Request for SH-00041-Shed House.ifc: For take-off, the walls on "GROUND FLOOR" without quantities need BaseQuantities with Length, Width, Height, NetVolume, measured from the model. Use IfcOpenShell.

First a look at what the model holds.

```python
import ifcopenshell
import ifcopenshell.util.element
import ifcopenshell.util.unit

model = ifcopenshell.open("SH-00041-Shed House.ifc")
print(model.schema)
for unit_type in ("LENGTHUNIT", "AREAUNIT", "VOLUMEUNIT"):
    print(unit_type, ifcopenshell.util.unit.calculate_unit_scale(model, unit_type))
storey = next(s for s in model.by_type("IfcBuildingStorey") if s.Name == "GROUND FLOOR")
walls = [e for e in ifcopenshell.util.element.get_decomposition(storey) if e.is_a("IfcWall")]
for e in sorted(walls, key=lambda e: e.id()):
    print(e.id(), e.is_a(), e.Name, list(ifcopenshell.util.element.get_psets(e, qtos_only=True)), sep=" | ")
```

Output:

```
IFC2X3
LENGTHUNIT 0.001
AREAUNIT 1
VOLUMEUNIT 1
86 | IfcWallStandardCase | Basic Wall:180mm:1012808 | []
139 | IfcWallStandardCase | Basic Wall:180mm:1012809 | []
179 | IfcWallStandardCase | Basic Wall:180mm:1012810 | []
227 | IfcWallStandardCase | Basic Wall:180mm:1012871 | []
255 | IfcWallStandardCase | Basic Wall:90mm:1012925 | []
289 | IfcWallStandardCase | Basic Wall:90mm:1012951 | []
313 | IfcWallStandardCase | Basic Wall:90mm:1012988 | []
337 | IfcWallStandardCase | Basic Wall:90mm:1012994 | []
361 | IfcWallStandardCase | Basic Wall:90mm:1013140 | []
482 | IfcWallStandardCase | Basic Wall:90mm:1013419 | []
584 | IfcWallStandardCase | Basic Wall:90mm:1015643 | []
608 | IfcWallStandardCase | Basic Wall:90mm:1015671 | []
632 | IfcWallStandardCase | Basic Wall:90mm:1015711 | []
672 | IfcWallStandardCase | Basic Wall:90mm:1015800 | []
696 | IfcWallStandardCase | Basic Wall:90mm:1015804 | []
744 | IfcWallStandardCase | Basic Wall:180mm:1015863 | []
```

```python
import ifcopenshell
import ifcopenshell.api.pset
import ifcopenshell.geom
import ifcopenshell.util.element
import ifcopenshell.util.shape
import ifcopenshell.util.unit

model = ifcopenshell.open("SH-00041-Shed House.ifc")
unit_scale = ifcopenshell.util.unit.calculate_unit_scale(model)
volume_scale = ifcopenshell.util.unit.calculate_unit_scale(model, "VOLUMEUNIT")
settings = ifcopenshell.geom.settings()

storey = next(s for s in model.by_type("IfcBuildingStorey") if s.Name == "GROUND FLOOR")
walls = [e for e in ifcopenshell.util.element.get_decomposition(storey) if e.is_a("IfcWall")]

for e in sorted(walls, key=lambda e: e.id()):
    if ifcopenshell.util.element.get_psets(e, qtos_only=True, should_inherit=False):
        continue
    # Geometry comes back in metres, in the element's own axes.
    shape = ifcopenshell.geom.create_shape(settings, e)
    values = {
        "Length": ifcopenshell.util.shape.get_x(shape.geometry) / unit_scale,
        "Width": ifcopenshell.util.shape.get_y(shape.geometry) / unit_scale,
        "Height": ifcopenshell.util.shape.get_z(shape.geometry) / unit_scale,
        "NetVolume": ifcopenshell.util.shape.get_volume(shape.geometry) / volume_scale,
    }
    qto = ifcopenshell.api.pset.add_qto(model, product=e, name="BaseQuantities")
    ifcopenshell.api.pset.edit_qto(model, qto=qto, properties=values)
    print(e.id(), {k: round(v, 3) for k, v in values.items()})

model.write("SH-00041-Shed House-out.ifc")
```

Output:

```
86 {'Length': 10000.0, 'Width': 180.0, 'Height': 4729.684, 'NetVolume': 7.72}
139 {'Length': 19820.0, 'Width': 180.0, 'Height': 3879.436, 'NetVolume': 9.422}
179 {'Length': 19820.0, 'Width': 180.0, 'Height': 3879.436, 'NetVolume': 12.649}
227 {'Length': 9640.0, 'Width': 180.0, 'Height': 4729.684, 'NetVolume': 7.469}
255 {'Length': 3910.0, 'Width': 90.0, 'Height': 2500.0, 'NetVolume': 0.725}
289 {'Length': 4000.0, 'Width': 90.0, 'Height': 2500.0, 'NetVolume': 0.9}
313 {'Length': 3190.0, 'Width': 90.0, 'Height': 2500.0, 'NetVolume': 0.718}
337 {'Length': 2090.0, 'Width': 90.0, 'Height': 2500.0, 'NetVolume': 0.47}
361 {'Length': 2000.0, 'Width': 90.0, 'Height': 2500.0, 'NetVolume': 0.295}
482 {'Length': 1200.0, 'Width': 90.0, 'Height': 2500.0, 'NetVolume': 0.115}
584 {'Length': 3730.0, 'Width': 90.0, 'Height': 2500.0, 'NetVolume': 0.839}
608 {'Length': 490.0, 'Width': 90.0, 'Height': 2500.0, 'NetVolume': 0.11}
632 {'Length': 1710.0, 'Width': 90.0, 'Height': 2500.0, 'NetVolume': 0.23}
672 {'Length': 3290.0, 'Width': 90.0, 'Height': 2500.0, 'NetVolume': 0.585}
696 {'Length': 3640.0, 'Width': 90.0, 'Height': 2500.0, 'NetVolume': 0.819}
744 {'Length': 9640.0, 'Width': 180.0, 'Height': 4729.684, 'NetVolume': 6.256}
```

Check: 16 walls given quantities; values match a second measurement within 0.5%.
